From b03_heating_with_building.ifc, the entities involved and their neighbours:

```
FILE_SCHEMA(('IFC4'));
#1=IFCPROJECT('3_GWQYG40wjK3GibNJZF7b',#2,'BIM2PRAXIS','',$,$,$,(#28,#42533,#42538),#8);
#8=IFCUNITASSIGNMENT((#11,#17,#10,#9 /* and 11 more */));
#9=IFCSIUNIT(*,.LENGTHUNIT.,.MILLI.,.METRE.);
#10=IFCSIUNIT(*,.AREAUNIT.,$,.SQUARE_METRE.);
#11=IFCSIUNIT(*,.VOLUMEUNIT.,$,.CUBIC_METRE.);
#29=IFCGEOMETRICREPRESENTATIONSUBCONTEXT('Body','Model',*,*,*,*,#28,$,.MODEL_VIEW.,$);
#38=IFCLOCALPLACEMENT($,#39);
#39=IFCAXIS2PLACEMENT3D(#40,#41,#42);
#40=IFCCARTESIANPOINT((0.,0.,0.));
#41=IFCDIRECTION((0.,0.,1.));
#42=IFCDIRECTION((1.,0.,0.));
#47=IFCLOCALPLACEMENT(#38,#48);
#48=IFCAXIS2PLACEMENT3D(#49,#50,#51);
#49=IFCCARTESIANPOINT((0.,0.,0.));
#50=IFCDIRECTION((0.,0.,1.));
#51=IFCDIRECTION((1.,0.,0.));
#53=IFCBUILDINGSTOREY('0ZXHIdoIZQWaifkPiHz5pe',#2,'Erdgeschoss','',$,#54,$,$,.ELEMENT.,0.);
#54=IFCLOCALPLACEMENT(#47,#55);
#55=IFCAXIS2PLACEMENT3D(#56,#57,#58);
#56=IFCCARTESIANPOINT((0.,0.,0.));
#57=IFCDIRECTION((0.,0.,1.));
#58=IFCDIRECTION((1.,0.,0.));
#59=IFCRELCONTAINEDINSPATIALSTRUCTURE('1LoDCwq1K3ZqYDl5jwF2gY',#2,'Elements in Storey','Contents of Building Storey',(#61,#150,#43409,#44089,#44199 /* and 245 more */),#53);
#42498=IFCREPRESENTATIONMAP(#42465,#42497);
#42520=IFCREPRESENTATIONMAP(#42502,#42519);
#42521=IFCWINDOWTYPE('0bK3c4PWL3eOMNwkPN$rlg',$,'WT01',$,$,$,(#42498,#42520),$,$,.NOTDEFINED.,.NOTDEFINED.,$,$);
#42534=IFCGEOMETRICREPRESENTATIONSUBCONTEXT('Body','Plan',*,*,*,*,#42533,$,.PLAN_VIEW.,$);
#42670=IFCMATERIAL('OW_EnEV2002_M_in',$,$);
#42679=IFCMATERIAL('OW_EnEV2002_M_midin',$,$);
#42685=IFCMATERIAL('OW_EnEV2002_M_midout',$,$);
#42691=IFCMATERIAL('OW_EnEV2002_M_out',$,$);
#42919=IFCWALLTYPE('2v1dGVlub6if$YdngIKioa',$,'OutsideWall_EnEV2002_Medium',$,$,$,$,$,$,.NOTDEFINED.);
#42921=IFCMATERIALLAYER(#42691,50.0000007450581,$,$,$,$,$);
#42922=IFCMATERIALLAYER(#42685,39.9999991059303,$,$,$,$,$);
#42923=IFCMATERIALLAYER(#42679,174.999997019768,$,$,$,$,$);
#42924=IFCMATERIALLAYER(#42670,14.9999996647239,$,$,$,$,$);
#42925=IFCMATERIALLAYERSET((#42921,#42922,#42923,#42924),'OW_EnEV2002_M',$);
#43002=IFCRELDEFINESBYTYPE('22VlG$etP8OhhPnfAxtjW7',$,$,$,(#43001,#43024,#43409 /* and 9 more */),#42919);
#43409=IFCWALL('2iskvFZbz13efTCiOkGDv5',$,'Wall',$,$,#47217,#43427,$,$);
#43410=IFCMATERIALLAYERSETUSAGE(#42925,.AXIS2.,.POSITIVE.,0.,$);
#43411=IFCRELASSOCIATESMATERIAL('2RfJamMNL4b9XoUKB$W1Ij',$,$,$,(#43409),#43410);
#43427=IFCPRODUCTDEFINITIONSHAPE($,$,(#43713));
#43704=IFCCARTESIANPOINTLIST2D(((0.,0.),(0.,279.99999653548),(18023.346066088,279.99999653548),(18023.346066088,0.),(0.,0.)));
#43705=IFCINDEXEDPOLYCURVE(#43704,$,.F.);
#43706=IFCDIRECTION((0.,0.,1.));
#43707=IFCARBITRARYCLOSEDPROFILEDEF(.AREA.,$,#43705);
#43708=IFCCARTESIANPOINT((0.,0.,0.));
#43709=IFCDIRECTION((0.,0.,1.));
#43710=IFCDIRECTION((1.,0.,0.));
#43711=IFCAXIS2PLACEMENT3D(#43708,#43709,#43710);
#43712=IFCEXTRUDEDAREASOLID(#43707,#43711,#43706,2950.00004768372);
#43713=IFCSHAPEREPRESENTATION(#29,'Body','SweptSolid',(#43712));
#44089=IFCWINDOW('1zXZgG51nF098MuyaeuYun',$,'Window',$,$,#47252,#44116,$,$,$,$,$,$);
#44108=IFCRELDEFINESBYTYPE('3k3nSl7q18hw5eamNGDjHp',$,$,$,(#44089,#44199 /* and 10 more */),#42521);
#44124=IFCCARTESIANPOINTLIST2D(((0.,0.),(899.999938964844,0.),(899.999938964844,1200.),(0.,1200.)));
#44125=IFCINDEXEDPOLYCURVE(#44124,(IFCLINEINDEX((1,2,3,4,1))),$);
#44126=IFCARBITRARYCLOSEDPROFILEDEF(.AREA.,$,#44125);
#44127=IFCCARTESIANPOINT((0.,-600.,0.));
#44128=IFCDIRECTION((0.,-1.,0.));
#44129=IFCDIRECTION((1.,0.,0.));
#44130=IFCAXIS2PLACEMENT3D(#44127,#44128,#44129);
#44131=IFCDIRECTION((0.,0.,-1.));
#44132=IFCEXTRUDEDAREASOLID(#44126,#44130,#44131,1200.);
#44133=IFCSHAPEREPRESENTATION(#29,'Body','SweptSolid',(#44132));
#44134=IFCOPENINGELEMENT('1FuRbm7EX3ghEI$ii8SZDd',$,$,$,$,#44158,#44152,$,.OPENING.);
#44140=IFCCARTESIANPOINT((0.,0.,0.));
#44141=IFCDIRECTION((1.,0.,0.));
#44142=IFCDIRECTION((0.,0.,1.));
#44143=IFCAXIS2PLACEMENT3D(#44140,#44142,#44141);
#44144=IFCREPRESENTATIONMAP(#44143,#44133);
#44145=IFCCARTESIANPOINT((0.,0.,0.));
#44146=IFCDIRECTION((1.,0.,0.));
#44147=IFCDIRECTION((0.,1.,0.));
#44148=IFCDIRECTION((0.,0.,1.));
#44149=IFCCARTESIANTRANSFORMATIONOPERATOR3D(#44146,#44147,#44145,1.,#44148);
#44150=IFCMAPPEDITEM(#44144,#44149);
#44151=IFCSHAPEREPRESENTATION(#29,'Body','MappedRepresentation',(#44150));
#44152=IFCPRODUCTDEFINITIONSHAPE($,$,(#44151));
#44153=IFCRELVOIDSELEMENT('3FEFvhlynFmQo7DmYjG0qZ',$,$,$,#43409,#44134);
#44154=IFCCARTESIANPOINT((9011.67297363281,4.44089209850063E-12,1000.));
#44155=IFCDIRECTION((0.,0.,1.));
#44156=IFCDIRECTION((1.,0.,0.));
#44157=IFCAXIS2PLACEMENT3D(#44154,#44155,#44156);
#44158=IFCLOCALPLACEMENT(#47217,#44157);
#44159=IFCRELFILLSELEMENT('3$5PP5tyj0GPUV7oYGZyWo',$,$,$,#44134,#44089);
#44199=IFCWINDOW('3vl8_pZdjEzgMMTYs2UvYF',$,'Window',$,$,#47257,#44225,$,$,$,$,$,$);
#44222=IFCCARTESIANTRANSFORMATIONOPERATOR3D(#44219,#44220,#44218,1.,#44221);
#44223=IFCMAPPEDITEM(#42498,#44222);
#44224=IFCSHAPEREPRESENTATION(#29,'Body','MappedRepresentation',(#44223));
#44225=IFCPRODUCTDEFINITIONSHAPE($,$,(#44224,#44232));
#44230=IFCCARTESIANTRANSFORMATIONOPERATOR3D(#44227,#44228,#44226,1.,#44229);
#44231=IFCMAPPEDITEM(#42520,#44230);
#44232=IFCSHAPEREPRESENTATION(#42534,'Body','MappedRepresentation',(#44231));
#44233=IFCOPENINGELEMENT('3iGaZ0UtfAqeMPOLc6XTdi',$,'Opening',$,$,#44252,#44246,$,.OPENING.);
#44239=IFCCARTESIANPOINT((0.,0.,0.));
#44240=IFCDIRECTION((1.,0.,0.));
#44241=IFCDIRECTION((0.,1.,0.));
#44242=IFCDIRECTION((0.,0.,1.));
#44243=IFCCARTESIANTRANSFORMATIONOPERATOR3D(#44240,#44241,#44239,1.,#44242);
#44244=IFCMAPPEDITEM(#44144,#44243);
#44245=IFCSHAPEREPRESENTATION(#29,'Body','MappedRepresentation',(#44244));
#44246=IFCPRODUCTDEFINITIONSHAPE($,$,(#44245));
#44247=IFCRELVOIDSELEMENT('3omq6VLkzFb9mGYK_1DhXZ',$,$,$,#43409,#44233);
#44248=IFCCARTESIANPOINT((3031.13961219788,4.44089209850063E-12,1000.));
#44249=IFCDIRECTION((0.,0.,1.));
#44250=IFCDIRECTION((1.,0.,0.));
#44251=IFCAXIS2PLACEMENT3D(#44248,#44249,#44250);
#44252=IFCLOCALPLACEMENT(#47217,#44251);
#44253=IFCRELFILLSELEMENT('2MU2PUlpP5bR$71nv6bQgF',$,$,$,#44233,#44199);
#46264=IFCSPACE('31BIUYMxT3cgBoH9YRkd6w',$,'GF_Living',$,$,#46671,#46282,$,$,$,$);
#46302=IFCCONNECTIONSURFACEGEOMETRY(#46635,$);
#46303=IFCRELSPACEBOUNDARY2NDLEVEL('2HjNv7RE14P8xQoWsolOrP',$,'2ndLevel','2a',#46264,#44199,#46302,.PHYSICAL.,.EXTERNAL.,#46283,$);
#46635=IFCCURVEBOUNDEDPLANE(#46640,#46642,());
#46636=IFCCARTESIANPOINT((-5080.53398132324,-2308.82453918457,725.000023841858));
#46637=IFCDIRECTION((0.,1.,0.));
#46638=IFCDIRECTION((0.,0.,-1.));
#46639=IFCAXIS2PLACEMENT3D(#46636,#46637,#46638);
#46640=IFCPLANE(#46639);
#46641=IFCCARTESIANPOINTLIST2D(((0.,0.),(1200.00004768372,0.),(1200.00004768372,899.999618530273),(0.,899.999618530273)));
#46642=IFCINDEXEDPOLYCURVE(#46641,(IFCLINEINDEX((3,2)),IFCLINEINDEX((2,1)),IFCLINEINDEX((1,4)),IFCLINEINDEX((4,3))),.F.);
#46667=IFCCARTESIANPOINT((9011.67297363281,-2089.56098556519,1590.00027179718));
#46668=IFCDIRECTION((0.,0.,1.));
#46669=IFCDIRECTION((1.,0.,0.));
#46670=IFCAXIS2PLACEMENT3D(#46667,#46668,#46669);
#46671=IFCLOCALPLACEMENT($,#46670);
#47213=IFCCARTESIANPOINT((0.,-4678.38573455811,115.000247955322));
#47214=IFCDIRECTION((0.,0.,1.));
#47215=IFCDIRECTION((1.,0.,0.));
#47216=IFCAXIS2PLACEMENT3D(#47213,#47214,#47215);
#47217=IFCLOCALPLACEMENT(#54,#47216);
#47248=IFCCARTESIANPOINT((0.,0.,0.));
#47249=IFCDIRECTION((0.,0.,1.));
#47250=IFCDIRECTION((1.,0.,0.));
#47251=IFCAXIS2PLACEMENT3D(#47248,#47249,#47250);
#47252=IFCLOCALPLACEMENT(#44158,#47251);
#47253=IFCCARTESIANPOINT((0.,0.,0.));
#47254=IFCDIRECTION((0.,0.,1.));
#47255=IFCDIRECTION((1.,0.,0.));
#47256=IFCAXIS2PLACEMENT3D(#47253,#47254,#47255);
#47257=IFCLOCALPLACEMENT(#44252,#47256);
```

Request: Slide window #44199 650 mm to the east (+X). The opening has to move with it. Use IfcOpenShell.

```python
import numpy as np
import ifcopenshell
import ifcopenshell.api.geometry
import ifcopenshell.util.placement

model = ifcopenshell.open("b03_heating_with_building.ifc")

window = model.by_guid("3vl8_pZdjEzgMMTYs2UvYF")
opening = window.FillsVoids[0].RelatingOpeningElement
wall = opening.VoidsElements[0].RelatingBuildingElement

wall_matrix = ifcopenshell.util.placement.get_local_placement(wall.ObjectPlacement)
shift = wall_matrix[:3, 0] * 650.0
before = ifcopenshell.util.placement.get_local_placement(window.ObjectPlacement)[:3, 3].copy()

# The window is placed relative to its opening, so it follows when the opening moves.
matrix = ifcopenshell.util.placement.get_local_placement(opening.ObjectPlacement)
matrix[:3, 3] += shift
ifcopenshell.api.geometry.edit_object_placement(
    model, product=opening, matrix=matrix, is_si=False, should_transform_children=True
)

# Space boundary surfaces are stored in each space's coordinates; move them too.
for rel in window.ProvidesBoundaries:
    if not rel.ConnectionGeometry:
        continue
    surface = rel.ConnectionGeometry.SurfaceOnRelatingElement.BasisSurface
    space_matrix = ifcopenshell.util.placement.get_local_placement(rel.RelatingSpace.ObjectPlacement)
    point = np.array(surface.Position.Location.Coordinates) + space_matrix[:3, :3].T @ shift
    surface.Position = model.createIfcAxis2Placement3D(
        model.createIfcCartesianPoint(point.tolist()), surface.Position.Axis, surface.Position.RefDirection
    )

after = ifcopenshell.util.placement.get_local_placement(window.ObjectPlacement)[:3, 3]
print("window moved by", (after - before).round(3) + 0.0)

model.write("b03_heating_with_building_edited.ifc")
```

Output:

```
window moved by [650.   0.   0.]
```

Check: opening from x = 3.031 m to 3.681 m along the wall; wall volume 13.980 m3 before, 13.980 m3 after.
